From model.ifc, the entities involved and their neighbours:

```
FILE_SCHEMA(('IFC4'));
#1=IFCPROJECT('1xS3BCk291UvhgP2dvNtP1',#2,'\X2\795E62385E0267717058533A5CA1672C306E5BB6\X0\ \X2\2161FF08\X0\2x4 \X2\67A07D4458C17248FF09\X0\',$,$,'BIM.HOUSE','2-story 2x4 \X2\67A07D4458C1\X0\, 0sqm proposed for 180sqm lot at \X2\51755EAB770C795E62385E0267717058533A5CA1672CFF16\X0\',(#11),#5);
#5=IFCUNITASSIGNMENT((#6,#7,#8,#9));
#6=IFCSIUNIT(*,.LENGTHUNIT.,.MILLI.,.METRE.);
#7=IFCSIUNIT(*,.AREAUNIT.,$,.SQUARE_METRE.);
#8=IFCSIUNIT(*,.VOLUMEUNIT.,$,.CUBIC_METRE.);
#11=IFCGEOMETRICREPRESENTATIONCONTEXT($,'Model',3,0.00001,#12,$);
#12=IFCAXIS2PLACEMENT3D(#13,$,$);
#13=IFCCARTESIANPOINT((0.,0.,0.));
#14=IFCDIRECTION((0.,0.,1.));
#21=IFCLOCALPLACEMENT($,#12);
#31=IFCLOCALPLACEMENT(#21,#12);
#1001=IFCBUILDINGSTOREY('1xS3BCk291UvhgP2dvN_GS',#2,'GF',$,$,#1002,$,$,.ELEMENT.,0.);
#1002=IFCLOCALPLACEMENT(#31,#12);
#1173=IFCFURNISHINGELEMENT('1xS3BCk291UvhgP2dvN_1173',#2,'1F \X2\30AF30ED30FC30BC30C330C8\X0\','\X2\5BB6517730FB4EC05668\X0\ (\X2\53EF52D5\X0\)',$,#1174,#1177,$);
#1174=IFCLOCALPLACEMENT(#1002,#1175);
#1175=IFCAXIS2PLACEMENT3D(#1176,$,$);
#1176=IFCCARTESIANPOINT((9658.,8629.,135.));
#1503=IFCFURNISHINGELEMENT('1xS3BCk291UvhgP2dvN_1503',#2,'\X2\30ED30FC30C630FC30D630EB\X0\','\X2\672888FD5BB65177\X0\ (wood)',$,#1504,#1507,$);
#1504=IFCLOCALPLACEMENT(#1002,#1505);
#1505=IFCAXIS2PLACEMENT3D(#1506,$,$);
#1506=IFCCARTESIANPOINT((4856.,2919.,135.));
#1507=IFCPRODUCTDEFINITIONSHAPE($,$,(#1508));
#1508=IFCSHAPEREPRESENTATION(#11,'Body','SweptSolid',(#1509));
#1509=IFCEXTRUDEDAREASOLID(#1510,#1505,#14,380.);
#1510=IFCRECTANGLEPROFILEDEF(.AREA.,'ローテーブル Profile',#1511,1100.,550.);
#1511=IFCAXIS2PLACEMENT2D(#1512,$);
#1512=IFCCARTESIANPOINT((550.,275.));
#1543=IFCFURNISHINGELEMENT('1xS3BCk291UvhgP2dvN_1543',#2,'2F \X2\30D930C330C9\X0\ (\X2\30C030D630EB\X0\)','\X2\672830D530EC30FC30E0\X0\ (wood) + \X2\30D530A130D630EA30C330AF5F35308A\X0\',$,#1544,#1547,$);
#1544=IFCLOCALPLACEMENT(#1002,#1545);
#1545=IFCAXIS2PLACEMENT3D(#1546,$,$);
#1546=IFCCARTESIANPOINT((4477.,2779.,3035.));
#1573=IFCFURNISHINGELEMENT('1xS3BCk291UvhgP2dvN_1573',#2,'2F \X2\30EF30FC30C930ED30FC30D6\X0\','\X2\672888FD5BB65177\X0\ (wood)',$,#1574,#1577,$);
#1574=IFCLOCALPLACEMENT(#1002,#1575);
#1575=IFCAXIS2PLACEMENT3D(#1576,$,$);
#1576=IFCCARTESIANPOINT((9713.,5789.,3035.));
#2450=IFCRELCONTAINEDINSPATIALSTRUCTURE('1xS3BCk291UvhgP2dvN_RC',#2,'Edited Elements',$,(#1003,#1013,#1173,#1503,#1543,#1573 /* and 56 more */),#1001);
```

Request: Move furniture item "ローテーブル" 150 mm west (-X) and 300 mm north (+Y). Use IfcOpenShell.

```python
import ifcopenshell
import ifcopenshell.api.geometry
import ifcopenshell.util.placement

model = ifcopenshell.open("model.ifc")

item = model.by_guid("1xS3BCk291UvhgP2dvN_1503")
matrix = ifcopenshell.util.placement.get_local_placement(item.ObjectPlacement)
matrix[0, 3] -= 150.0
matrix[1, 3] += 300.0
ifcopenshell.api.geometry.edit_object_placement(model, product=item, matrix=matrix, is_si=False)

print(ifcopenshell.util.placement.get_local_placement(item.ObjectPlacement).round(3) + 0.0)

model.write("model_updated.ifc")
```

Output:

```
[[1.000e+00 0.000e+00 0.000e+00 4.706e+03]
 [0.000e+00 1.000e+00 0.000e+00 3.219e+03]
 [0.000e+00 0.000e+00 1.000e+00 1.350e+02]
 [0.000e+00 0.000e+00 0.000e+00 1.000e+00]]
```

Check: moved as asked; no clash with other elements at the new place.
